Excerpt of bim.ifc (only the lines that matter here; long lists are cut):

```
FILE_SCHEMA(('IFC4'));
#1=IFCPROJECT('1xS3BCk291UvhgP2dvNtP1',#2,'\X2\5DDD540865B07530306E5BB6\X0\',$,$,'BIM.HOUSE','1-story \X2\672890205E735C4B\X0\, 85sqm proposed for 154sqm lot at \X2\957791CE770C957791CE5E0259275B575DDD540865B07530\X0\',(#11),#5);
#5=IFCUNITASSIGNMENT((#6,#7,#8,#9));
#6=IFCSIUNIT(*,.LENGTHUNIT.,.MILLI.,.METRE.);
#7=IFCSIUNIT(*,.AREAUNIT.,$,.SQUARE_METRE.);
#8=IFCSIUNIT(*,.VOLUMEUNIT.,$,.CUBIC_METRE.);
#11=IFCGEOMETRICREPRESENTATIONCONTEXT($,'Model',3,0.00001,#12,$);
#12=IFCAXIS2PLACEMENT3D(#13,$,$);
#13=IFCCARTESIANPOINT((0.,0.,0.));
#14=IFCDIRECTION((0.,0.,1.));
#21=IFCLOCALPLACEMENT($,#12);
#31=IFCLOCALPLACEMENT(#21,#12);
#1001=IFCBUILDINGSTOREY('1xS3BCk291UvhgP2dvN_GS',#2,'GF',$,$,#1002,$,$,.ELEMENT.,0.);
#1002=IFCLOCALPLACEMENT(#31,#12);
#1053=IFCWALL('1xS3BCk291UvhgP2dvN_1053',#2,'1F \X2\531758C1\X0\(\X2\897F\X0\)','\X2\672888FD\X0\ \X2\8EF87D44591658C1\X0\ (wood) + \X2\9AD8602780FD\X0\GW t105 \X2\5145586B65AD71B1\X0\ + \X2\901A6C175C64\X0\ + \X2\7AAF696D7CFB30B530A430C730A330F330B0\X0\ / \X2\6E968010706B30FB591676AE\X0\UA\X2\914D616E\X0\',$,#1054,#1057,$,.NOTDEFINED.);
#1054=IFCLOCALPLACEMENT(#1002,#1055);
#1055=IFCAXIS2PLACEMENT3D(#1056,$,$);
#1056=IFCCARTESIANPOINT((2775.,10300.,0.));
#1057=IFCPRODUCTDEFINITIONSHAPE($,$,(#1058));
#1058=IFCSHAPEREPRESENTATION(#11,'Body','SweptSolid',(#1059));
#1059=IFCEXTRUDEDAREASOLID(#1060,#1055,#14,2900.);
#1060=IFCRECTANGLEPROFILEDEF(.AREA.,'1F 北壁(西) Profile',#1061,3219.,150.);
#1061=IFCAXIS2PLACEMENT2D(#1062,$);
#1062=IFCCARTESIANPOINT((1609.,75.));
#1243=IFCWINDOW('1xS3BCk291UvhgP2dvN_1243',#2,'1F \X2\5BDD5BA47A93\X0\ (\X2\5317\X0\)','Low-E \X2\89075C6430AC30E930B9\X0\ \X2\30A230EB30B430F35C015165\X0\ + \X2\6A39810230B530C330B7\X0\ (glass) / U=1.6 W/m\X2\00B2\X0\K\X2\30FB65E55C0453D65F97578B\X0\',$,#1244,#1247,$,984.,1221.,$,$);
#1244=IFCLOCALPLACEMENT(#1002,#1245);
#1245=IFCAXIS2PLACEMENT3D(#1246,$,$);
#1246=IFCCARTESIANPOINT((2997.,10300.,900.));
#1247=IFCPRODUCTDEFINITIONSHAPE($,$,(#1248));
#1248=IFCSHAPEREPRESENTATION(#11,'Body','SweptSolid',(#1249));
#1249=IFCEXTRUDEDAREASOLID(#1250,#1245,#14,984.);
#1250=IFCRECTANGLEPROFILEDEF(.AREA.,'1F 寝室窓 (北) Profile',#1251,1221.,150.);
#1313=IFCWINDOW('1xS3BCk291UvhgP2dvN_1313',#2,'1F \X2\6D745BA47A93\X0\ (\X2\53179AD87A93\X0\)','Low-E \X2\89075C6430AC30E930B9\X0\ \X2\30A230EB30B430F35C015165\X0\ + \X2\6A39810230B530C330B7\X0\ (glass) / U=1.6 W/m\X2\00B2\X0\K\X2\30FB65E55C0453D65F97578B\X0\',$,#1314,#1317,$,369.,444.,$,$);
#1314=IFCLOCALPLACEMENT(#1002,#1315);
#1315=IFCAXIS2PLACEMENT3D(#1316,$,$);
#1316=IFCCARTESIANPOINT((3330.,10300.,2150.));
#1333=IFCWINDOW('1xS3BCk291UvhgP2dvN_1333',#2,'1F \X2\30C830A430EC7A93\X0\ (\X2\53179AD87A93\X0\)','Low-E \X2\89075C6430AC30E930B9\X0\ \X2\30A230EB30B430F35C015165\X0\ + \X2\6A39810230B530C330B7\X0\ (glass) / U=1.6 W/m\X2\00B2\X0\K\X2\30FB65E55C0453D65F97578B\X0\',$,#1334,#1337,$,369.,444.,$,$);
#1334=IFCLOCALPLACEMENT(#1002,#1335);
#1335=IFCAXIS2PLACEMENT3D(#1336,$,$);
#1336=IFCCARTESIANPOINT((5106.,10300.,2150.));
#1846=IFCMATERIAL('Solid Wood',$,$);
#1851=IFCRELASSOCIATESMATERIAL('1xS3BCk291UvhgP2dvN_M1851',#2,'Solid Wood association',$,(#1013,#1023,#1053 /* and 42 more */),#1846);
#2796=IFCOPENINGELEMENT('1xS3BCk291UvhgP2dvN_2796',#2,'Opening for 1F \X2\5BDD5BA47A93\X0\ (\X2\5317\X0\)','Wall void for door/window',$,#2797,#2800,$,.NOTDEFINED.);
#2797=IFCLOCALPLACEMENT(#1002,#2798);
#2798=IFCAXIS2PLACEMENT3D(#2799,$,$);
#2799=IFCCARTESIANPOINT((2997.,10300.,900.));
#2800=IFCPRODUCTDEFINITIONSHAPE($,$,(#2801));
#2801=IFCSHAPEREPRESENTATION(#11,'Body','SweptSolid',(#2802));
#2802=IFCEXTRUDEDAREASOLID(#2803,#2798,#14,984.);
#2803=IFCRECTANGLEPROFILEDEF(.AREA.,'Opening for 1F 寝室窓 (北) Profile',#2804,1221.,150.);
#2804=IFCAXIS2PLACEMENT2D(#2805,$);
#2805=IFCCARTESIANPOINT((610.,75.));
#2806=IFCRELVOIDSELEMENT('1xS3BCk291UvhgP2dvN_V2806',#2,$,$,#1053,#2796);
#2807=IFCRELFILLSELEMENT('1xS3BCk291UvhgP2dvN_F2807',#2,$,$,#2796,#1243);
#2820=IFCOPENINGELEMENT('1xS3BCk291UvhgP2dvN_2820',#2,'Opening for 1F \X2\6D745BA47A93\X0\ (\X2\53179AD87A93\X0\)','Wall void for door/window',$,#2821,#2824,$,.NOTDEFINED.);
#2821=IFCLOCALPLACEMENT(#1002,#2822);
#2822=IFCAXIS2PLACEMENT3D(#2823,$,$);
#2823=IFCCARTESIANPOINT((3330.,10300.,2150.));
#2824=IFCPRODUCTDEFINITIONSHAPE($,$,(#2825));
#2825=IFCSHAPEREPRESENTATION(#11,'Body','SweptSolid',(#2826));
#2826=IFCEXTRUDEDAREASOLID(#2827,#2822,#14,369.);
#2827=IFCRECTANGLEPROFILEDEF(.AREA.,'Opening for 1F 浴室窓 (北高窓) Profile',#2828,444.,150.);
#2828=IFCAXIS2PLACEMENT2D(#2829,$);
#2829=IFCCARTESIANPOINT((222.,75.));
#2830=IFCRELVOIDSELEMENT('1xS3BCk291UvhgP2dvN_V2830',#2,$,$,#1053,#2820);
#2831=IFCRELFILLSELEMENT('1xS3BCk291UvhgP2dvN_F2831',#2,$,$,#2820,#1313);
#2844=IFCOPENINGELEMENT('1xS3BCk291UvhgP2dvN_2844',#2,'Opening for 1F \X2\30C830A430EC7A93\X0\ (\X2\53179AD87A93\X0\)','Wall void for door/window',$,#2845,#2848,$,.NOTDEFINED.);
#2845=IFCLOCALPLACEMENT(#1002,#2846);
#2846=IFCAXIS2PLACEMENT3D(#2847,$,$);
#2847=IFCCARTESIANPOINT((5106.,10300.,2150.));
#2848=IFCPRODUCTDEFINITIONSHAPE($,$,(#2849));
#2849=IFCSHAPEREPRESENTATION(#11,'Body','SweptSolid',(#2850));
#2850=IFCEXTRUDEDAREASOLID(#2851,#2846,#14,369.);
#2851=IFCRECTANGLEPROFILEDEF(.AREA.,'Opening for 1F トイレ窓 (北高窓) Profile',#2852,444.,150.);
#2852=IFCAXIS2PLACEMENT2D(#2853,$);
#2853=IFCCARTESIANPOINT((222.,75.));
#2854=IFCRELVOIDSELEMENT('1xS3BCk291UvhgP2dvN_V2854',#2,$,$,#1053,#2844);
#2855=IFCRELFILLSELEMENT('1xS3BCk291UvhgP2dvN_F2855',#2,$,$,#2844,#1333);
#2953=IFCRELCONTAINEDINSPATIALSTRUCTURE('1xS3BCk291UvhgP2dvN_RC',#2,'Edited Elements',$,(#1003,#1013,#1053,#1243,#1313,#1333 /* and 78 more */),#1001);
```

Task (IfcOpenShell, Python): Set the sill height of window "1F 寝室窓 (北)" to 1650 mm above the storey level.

```python
import numpy as np
import ifcopenshell
import ifcopenshell.api.geometry
import ifcopenshell.geom
import ifcopenshell.util.element
import ifcopenshell.util.placement
import ifcopenshell.util.shape
import ifcopenshell.util.unit

model = ifcopenshell.open("bim.ifc")
unit_scale = ifcopenshell.util.unit.calculate_unit_scale(model)

window = model.by_guid("1xS3BCk291UvhgP2dvN_1243")
opening = window.FillsVoids[0].RelatingOpeningElement
storey = ifcopenshell.util.element.get_container(window, ifc_class="IfcBuildingStorey")
level = ifcopenshell.util.placement.get_local_placement(storey.ObjectPlacement)[2, 3]

# The opening's origin need not be at the sill, so measure its lowest point.
shape = ifcopenshell.geom.create_shape(ifcopenshell.geom.settings(), opening)
bottom = ifcopenshell.util.shape.get_shape_bottom_elevation(shape, shape.geometry) / unit_scale
dz = level + 1.65 / unit_scale - bottom

shift = np.array([0.0, 0.0, dz])
# The window is not placed relative to its opening, so move both.
for product in (opening, window):
    matrix = ifcopenshell.util.placement.get_local_placement(product.ObjectPlacement)
    matrix[:3, 3] += shift
    ifcopenshell.api.geometry.edit_object_placement(model, product=product, matrix=matrix, is_si=False)

print(f"moved by {dz * unit_scale:+.3f} m")

model.write("bim_updated.ifc")
```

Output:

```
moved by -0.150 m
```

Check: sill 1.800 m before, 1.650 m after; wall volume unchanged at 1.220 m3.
